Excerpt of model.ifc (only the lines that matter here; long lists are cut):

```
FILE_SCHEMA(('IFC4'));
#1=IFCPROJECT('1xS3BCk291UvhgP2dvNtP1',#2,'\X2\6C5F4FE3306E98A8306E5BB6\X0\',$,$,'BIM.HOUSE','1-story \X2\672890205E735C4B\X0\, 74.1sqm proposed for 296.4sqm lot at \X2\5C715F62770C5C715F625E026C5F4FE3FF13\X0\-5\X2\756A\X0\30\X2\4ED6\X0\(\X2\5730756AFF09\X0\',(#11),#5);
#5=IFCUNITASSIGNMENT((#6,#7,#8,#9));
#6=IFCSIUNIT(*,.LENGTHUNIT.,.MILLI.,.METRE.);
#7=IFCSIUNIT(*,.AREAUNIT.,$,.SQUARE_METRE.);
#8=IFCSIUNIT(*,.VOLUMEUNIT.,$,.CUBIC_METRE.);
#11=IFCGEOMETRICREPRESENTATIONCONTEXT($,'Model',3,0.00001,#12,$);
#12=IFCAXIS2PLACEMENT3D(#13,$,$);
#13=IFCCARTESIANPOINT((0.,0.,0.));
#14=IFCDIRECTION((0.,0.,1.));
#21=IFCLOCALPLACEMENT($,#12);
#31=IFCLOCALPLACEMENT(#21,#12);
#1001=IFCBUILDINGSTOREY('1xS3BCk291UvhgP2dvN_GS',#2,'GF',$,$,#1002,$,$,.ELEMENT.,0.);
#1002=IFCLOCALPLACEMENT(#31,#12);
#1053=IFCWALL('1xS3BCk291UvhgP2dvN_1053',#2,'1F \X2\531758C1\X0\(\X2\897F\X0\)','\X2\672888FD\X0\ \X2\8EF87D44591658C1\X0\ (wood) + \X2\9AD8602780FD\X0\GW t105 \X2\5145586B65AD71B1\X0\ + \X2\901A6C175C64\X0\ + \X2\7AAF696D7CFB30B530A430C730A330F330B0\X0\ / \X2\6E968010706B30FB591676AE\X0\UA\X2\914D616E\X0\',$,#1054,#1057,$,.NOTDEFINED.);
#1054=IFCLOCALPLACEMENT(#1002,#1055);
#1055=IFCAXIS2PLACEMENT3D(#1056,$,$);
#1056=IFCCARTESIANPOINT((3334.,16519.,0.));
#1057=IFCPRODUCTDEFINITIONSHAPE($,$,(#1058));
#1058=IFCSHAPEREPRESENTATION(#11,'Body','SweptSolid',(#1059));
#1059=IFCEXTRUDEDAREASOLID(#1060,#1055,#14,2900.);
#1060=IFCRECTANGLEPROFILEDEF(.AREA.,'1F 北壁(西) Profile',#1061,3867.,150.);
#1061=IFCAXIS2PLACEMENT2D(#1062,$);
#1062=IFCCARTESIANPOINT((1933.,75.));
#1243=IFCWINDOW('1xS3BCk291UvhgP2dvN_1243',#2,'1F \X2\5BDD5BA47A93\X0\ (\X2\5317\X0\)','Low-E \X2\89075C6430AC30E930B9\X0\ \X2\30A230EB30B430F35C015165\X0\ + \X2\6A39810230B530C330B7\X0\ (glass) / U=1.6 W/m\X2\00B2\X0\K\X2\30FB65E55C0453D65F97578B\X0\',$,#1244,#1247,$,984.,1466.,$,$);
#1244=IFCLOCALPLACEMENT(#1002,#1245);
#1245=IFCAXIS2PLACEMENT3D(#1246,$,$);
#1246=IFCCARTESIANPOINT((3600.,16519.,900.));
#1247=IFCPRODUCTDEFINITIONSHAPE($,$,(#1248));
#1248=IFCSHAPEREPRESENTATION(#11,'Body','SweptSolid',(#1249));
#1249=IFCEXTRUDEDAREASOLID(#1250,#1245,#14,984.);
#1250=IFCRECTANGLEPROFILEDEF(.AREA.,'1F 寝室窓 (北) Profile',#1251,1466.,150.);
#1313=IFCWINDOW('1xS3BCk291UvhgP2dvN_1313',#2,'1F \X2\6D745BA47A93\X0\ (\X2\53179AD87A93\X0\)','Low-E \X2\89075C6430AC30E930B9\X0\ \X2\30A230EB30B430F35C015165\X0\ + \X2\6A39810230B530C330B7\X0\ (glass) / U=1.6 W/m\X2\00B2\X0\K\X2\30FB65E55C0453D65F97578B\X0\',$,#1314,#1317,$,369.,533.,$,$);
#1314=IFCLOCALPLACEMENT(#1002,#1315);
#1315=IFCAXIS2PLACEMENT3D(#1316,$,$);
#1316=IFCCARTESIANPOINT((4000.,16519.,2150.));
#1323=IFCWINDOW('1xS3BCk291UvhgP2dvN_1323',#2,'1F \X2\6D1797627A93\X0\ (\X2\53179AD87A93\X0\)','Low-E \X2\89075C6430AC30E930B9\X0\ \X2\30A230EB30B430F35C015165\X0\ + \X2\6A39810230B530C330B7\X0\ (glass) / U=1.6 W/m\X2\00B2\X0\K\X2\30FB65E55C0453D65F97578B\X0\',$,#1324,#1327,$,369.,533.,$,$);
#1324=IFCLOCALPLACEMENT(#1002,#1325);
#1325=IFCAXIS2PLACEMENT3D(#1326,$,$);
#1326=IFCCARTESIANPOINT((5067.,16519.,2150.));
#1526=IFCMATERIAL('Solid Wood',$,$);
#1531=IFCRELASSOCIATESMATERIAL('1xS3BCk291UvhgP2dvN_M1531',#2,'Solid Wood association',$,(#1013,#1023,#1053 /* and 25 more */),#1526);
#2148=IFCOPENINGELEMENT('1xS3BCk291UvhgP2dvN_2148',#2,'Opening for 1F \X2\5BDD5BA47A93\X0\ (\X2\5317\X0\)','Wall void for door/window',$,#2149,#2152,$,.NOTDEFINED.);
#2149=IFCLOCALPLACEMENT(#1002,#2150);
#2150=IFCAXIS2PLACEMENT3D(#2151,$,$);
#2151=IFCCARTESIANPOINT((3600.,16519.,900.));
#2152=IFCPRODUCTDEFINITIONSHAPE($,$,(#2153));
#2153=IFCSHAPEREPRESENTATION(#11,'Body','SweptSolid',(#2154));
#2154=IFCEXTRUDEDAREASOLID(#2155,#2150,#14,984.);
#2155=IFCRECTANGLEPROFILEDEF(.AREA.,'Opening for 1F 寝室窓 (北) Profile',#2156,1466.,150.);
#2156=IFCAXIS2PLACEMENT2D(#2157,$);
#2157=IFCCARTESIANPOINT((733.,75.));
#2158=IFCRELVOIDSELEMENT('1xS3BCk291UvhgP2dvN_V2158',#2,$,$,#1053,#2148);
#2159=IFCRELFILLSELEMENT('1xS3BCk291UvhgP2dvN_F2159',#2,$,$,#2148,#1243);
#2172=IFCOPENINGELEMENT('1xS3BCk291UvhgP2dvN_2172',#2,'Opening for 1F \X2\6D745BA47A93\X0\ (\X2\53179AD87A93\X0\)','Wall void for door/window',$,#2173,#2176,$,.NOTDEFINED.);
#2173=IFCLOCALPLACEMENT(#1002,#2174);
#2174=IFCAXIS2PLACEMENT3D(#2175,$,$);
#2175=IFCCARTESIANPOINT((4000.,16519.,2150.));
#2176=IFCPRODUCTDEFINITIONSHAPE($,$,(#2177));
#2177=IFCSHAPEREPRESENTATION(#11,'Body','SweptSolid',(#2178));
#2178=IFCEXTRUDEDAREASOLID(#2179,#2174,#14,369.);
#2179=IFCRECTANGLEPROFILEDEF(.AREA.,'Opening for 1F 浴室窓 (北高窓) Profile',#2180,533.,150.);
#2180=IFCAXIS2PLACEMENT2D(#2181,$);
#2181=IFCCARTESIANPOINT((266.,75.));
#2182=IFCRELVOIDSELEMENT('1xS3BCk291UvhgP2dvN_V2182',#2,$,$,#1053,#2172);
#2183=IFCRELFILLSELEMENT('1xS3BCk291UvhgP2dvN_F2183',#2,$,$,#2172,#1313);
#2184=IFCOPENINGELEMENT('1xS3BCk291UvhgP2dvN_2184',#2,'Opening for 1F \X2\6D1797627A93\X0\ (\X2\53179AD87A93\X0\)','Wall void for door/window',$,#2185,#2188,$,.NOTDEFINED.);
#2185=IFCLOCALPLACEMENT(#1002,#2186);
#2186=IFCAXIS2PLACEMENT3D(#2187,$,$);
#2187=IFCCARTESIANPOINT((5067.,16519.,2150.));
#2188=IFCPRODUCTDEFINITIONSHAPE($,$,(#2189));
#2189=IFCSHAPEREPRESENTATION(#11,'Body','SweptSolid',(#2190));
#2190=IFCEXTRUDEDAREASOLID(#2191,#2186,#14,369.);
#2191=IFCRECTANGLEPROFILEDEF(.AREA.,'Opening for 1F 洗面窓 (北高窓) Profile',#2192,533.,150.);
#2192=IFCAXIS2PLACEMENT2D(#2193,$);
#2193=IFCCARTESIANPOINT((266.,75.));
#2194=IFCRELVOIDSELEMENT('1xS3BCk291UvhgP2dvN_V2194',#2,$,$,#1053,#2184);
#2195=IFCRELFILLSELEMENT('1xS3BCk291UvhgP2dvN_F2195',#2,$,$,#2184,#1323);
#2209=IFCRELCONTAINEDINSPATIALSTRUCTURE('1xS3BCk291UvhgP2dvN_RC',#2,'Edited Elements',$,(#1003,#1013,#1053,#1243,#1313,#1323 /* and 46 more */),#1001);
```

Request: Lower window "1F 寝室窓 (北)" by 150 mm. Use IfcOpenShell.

```python
import numpy as np
import ifcopenshell
import ifcopenshell.api.geometry
import ifcopenshell.util.placement
import ifcopenshell.util.unit

model = ifcopenshell.open("model.ifc")
unit_scale = ifcopenshell.util.unit.calculate_unit_scale(model)

window = model.by_guid("1xS3BCk291UvhgP2dvN_1243")
opening = window.FillsVoids[0].RelatingOpeningElement
dz = -150.0

shift = np.array([0.0, 0.0, dz])
# The window is not placed relative to its opening, so move both.
for product in (opening, window):
    matrix = ifcopenshell.util.placement.get_local_placement(product.ObjectPlacement)
    matrix[:3, 3] += shift
    ifcopenshell.api.geometry.edit_object_placement(model, product=product, matrix=matrix, is_si=False)

print(f"moved by {dz * unit_scale:+.3f} m")

model.write("model_updated.ifc")
```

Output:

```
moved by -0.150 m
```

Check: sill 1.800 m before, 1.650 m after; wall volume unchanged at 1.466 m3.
